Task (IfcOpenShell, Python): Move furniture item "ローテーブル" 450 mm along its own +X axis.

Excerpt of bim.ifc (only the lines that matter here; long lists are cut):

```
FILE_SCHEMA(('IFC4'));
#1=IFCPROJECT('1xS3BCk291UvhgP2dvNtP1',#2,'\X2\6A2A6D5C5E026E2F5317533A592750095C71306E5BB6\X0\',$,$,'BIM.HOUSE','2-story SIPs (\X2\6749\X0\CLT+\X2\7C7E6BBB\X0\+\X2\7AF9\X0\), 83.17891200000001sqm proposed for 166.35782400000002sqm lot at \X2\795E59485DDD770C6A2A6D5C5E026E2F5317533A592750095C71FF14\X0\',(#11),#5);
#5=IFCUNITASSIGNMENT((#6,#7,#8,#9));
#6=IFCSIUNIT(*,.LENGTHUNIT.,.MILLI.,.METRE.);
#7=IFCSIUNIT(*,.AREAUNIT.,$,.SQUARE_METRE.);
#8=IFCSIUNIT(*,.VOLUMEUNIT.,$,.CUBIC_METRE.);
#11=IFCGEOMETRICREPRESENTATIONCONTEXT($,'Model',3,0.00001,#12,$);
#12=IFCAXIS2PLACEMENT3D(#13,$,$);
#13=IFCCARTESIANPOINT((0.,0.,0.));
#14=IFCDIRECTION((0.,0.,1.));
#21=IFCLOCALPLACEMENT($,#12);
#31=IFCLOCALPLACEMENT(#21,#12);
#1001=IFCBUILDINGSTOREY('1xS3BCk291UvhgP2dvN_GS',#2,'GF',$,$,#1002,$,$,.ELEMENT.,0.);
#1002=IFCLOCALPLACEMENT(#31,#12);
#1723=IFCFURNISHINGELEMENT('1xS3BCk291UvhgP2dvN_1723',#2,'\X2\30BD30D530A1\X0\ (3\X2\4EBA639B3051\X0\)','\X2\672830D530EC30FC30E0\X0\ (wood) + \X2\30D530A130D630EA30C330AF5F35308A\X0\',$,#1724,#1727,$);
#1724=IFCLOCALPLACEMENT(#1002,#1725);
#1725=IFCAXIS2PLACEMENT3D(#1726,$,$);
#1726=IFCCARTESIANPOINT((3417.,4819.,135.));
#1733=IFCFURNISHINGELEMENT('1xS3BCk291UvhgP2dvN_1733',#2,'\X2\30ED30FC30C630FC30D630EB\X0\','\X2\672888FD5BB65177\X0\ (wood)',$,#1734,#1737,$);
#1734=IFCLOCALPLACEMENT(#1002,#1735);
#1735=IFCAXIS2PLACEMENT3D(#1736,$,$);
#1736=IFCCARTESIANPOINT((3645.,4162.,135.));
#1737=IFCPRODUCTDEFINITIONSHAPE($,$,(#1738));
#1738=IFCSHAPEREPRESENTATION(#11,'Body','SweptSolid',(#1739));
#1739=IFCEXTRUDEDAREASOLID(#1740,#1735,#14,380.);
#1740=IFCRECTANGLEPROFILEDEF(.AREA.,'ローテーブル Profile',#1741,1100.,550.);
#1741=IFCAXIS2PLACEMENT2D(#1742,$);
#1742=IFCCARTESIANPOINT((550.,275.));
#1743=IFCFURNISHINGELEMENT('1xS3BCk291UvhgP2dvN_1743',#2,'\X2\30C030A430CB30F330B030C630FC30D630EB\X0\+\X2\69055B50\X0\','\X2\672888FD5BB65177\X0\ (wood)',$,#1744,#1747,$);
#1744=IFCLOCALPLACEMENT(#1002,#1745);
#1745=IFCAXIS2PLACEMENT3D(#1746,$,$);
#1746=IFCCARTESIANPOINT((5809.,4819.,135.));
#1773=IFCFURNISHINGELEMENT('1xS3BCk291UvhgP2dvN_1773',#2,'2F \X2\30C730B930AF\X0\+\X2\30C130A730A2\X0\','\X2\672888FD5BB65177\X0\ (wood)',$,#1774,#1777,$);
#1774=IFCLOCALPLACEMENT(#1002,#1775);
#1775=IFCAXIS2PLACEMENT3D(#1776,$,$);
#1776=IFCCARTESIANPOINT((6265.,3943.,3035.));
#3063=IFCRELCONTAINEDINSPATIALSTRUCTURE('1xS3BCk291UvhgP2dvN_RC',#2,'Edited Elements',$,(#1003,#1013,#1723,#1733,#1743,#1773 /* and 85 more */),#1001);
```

```python
import ifcopenshell
import ifcopenshell.api.geometry
import ifcopenshell.util.placement
import ifcopenshell.util.unit

model = ifcopenshell.open("bim.ifc")
unit_scale = ifcopenshell.util.unit.calculate_unit_scale(model)

item = model.by_guid("1xS3BCk291UvhgP2dvN_1733")
matrix = ifcopenshell.util.placement.get_local_placement(item.ObjectPlacement)
matrix[:3, 3] += matrix[:3, 0] * 0.45 / unit_scale
ifcopenshell.api.geometry.edit_object_placement(model, product=item, matrix=matrix, is_si=False)

print(ifcopenshell.util.placement.get_local_placement(item.ObjectPlacement).round(3) + 0.0)

model.write("bim-out.ifc")
```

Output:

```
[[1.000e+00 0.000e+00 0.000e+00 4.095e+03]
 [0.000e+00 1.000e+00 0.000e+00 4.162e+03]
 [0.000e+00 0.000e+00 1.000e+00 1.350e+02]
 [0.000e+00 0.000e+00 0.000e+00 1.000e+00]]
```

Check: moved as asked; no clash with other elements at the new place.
